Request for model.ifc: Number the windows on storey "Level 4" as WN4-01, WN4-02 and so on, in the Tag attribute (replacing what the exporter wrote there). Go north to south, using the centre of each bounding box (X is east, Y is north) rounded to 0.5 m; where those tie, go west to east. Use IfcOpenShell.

First a look at what the model holds.

```python
import ifcopenshell
import ifcopenshell.util.element
import ifcopenshell.util.placement

model = ifcopenshell.open("model.ifc")
print(model.schema)
storey = next(s for s in model.by_type("IfcBuildingStorey") if s.Name == "Level 4")
windows = [e for e in ifcopenshell.util.element.get_decomposition(storey) if e.is_a("IfcWindow")]
for e in sorted(windows, key=lambda e: e.id()):
    origin = ifcopenshell.util.placement.get_local_placement(e.ObjectPlacement)[:3, 3]
    print(e.id(), e.Tag, e.Name, origin.round(2) + 0.0, sep=" | ")
```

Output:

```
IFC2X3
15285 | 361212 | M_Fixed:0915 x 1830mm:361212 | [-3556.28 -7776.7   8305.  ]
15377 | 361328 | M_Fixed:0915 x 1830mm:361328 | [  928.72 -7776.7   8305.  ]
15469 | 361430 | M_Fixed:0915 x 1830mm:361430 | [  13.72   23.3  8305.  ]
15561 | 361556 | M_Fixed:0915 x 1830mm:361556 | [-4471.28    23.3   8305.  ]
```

```python
import ifcopenshell
import ifcopenshell.geom
import ifcopenshell.util.element
import ifcopenshell.util.shape

model = ifcopenshell.open("model.ifc")
settings = ifcopenshell.geom.settings()
settings.set("use-world-coords", True)


def centre(element):
    shape = ifcopenshell.geom.create_shape(settings, element)
    return ifcopenshell.util.shape.get_bbox_centroid(shape.geometry)


storey = next(s for s in model.by_type("IfcBuildingStorey") if s.Name == "Level 4")
windows = [e for e in ifcopenshell.util.element.get_decomposition(storey) if e.is_a("IfcWindow")]

# Insertion points can sit at a corner or the storey origin, so sort by the geometry (in metres).
centres = {e: centre(e) for e in windows}
windows.sort(key=lambda e: (-round(centres[e][1] / 0.5), centres[e][0]))

for i, e in enumerate(windows, start=1):
    number = f"WN4-{i:02d}"
    e.Tag = number
    print(e.id(), number)

model.write("model_v2.ifc")
```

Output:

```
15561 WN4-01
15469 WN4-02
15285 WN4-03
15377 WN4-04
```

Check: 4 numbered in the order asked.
